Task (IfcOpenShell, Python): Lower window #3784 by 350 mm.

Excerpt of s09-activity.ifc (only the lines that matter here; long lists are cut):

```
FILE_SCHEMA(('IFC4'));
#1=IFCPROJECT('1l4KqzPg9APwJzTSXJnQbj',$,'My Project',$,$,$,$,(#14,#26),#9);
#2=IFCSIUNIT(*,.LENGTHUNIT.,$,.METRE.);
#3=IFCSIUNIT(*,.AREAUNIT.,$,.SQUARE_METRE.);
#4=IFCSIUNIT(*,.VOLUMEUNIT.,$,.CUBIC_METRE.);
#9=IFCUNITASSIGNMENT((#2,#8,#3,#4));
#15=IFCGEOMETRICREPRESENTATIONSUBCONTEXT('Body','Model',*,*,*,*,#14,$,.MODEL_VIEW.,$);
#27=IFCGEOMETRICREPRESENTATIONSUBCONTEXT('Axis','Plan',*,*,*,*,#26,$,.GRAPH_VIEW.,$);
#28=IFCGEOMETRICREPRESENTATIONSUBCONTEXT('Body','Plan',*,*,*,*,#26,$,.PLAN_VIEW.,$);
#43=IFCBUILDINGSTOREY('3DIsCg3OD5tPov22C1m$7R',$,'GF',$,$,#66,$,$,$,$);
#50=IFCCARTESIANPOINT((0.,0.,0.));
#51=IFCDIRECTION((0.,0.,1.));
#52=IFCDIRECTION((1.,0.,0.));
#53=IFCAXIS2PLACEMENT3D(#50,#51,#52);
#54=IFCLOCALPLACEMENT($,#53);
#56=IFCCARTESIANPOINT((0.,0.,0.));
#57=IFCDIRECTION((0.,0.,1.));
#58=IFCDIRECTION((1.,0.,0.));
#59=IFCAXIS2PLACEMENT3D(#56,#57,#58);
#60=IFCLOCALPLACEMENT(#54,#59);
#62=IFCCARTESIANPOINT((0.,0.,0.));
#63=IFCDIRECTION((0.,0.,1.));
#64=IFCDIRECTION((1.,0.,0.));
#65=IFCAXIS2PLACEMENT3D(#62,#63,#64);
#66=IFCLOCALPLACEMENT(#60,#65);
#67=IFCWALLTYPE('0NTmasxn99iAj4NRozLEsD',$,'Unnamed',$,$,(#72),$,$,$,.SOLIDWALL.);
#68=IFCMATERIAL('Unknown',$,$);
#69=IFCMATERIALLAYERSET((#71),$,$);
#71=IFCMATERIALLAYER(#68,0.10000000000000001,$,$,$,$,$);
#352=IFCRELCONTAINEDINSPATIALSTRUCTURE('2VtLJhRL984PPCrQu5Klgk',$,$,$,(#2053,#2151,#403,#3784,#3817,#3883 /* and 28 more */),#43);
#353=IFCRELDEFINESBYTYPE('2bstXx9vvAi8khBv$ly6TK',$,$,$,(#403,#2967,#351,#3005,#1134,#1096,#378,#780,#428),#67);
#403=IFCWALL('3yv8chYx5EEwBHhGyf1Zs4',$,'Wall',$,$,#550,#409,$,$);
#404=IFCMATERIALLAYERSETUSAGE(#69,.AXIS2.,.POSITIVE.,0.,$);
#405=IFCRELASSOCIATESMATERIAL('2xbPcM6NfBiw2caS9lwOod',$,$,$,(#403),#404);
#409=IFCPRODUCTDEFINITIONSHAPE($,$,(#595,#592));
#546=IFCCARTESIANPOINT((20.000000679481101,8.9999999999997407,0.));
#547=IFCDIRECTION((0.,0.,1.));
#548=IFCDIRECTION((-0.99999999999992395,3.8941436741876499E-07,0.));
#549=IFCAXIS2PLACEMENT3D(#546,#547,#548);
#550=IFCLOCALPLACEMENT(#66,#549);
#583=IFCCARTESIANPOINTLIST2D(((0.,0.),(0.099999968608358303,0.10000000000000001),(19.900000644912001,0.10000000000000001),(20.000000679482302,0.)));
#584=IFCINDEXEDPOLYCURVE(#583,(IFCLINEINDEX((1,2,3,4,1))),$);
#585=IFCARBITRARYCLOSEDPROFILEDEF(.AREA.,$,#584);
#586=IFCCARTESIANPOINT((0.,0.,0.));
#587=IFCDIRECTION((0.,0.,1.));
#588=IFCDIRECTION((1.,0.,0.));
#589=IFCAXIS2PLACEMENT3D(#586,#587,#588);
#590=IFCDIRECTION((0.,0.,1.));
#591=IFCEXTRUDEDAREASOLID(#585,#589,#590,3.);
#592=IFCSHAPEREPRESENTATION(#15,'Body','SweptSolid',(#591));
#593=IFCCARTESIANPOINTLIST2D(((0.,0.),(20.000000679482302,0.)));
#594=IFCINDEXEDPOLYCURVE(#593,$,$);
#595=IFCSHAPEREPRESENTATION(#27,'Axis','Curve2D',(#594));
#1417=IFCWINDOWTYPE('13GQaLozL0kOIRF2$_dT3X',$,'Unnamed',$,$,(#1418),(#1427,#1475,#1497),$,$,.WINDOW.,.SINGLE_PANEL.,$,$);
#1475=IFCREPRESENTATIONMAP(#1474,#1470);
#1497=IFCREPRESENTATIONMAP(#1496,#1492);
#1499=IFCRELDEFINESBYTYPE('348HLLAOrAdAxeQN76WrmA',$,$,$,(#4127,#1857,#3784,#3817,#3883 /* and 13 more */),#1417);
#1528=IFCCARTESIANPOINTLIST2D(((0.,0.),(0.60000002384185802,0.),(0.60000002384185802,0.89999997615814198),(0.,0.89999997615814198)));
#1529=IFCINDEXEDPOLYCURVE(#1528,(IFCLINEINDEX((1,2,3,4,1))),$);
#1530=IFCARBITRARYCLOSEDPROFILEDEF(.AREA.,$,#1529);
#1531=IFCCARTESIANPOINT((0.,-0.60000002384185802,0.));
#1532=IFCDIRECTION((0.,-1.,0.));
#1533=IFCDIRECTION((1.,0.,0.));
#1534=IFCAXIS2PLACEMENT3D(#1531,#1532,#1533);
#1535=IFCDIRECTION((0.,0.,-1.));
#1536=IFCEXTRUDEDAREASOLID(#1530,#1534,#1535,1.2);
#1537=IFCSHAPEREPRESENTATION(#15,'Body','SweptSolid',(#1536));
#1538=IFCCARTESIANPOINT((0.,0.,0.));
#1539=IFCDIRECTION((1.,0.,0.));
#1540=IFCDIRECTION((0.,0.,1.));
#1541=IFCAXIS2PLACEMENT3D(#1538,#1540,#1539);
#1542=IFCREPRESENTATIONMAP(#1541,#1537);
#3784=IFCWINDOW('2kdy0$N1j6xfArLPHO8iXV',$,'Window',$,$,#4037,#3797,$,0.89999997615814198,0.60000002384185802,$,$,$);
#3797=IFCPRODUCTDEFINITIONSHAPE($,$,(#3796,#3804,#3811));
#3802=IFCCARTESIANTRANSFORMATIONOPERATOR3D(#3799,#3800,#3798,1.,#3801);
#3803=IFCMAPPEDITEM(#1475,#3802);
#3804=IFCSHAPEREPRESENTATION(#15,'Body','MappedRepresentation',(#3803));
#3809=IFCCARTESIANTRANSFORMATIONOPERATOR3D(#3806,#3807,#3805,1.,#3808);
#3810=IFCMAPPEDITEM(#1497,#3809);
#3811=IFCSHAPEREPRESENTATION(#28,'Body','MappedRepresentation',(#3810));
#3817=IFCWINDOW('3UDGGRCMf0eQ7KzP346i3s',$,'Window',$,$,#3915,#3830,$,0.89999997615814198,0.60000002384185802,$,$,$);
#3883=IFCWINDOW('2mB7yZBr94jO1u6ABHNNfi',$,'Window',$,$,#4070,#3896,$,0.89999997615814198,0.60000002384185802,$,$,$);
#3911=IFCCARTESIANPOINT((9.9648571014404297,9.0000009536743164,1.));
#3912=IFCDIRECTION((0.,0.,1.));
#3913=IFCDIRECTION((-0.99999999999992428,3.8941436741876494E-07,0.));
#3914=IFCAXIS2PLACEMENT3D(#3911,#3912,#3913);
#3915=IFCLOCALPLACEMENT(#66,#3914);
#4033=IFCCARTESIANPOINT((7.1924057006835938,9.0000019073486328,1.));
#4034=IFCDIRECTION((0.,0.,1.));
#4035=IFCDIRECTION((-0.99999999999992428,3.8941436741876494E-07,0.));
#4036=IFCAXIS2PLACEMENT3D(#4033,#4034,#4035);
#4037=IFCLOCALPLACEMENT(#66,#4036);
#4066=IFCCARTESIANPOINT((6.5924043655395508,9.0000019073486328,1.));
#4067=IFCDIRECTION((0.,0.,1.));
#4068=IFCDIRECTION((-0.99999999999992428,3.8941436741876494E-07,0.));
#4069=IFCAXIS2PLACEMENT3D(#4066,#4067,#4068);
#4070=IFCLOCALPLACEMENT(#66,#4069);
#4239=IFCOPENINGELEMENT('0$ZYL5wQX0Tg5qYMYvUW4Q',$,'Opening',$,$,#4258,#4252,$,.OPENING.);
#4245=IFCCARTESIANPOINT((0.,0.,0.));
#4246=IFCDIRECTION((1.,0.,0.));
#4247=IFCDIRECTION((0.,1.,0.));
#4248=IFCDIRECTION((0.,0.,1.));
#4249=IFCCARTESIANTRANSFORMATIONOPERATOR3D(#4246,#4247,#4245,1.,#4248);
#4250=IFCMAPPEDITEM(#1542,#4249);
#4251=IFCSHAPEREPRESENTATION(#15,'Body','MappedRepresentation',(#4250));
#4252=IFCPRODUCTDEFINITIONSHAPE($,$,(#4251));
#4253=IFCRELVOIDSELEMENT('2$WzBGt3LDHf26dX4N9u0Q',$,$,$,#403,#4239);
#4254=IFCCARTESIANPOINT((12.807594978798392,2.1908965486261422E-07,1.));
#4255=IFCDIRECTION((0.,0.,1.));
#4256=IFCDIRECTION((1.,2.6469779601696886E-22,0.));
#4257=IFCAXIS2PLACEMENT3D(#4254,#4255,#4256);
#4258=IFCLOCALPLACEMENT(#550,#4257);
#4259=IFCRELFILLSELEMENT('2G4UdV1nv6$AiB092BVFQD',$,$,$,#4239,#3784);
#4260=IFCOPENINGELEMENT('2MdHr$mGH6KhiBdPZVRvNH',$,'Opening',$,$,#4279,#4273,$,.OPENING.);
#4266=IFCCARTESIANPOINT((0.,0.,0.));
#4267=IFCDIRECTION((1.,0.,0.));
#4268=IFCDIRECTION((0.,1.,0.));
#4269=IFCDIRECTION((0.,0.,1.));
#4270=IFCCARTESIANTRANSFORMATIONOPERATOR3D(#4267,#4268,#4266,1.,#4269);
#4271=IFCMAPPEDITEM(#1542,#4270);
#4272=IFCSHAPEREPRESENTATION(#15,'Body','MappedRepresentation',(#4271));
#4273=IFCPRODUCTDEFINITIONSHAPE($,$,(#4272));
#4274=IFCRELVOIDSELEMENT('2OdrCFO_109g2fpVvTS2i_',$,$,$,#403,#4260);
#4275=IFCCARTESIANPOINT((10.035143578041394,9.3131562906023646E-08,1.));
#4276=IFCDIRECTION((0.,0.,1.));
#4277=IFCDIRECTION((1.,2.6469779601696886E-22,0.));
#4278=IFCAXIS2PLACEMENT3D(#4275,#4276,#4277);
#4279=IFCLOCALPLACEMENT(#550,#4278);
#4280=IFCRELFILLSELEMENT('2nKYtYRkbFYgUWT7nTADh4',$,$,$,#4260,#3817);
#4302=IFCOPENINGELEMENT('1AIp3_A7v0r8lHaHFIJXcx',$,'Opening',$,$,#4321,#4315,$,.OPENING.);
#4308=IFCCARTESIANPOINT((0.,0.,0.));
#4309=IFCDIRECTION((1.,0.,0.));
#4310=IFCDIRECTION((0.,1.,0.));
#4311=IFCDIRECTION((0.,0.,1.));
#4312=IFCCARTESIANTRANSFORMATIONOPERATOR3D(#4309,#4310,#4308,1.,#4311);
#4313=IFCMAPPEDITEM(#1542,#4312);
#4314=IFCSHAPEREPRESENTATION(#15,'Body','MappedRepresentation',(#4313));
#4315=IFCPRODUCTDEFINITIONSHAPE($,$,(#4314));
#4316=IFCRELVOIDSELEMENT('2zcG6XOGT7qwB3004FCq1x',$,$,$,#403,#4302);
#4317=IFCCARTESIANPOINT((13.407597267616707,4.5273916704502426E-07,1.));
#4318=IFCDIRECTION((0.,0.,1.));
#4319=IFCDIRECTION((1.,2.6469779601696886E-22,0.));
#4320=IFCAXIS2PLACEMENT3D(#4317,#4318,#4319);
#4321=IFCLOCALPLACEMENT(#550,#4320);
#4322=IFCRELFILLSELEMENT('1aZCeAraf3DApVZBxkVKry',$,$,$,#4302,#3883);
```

```python
import numpy as np
import ifcopenshell
import ifcopenshell.api.geometry
import ifcopenshell.util.placement
import ifcopenshell.util.unit

model = ifcopenshell.open("s09-activity.ifc")
unit_scale = ifcopenshell.util.unit.calculate_unit_scale(model)

window = model.by_guid("2kdy0$N1j6xfArLPHO8iXV")
opening = window.FillsVoids[0].RelatingOpeningElement
dz = -0.35 / unit_scale

shift = np.array([0.0, 0.0, dz])
# The window is not placed relative to its opening, so move both.
for product in (opening, window):
    matrix = ifcopenshell.util.placement.get_local_placement(product.ObjectPlacement)
    matrix[:3, 3] += shift
    ifcopenshell.api.geometry.edit_object_placement(model, product=product, matrix=matrix, is_si=False)

print(f"moved by {dz * unit_scale:+.3f} m")

model.write("s09-activity_updated.ifc")
```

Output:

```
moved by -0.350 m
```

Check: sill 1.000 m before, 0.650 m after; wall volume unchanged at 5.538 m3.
